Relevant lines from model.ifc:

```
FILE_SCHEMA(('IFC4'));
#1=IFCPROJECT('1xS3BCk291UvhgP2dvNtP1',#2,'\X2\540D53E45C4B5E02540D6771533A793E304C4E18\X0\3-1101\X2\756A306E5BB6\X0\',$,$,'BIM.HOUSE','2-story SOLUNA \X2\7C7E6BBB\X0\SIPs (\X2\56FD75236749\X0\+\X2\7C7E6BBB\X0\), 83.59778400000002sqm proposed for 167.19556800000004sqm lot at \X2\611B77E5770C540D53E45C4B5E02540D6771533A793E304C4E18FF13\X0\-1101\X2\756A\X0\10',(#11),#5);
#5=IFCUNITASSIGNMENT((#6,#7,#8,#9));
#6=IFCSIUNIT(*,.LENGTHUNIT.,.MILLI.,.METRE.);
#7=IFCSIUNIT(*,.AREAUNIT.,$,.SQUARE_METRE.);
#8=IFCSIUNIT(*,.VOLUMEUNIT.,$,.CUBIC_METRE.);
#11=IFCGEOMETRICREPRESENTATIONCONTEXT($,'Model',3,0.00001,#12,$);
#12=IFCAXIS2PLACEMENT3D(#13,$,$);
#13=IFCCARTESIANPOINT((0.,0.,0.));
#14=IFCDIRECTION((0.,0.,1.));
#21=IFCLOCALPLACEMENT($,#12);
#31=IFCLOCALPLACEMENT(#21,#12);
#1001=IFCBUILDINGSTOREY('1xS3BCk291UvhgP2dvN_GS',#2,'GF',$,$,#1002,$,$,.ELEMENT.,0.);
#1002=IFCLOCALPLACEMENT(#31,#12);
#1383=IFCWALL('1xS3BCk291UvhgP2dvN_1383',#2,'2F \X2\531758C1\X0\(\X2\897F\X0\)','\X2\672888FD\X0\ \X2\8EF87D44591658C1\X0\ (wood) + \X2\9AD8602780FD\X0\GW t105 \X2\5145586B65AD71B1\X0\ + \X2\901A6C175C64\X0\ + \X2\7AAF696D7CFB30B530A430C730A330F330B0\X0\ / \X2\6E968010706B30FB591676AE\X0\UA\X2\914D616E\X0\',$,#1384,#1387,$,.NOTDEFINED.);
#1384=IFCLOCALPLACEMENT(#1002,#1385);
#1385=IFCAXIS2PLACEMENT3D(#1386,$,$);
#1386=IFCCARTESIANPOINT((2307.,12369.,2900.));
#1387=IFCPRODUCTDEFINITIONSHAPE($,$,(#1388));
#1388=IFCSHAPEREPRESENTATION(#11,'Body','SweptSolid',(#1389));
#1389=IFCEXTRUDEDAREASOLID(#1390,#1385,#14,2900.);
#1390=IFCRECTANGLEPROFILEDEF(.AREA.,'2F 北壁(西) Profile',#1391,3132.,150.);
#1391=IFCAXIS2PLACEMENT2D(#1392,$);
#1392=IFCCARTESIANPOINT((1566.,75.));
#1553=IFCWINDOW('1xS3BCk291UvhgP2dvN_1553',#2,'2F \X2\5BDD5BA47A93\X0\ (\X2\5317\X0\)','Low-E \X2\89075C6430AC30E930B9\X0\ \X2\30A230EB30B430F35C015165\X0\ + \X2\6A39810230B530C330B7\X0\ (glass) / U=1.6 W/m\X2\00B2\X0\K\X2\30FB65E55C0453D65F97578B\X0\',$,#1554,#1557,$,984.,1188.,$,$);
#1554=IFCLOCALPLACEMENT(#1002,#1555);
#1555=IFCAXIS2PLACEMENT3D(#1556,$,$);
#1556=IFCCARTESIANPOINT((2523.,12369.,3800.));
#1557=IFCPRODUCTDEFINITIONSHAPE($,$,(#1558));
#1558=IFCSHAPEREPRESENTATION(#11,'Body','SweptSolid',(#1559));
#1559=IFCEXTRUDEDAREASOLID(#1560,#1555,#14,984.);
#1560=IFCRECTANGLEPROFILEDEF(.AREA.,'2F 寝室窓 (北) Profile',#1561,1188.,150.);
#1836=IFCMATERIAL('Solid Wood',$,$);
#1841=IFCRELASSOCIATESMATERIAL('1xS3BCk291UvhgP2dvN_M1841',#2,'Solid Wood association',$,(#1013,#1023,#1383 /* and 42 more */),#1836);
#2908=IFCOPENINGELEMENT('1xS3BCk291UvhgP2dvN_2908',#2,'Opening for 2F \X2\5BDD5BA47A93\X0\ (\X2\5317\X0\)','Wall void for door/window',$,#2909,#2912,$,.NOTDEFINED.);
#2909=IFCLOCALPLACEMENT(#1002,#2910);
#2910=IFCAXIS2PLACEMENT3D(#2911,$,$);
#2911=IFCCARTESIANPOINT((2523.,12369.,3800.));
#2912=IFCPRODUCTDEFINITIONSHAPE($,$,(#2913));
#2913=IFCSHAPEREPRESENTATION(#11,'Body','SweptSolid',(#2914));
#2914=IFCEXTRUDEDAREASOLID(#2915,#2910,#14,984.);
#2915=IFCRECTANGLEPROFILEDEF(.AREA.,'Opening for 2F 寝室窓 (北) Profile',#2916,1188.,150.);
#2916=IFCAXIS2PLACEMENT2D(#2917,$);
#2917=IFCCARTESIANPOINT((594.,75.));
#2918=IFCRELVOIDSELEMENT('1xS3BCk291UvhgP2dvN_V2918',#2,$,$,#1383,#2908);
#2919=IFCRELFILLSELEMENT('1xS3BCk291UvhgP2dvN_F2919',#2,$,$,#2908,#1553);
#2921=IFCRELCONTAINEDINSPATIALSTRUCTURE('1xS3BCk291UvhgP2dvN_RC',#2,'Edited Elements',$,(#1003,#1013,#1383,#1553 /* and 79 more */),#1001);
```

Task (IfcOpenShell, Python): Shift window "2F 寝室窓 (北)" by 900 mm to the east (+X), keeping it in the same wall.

```python
import ifcopenshell
import ifcopenshell.api.geometry
import ifcopenshell.util.placement

model = ifcopenshell.open("model.ifc")

window = model.by_guid("1xS3BCk291UvhgP2dvN_1553")
opening = window.FillsVoids[0].RelatingOpeningElement
wall = opening.VoidsElements[0].RelatingBuildingElement

wall_matrix = ifcopenshell.util.placement.get_local_placement(wall.ObjectPlacement)
shift = wall_matrix[:3, 0] * 900.0
before = ifcopenshell.util.placement.get_local_placement(window.ObjectPlacement)[:3, 3].copy()

# The window is not placed relative to its opening, so move both.
for product in (opening, window):
    matrix = ifcopenshell.util.placement.get_local_placement(product.ObjectPlacement)
    matrix[:3, 3] += shift
    ifcopenshell.api.geometry.edit_object_placement(model, product=product, matrix=matrix, is_si=False)

after = ifcopenshell.util.placement.get_local_placement(window.ObjectPlacement)[:3, 3]
print("window moved by", (after - before).round(3) + 0.0)

model.write("model_rev.ifc")
```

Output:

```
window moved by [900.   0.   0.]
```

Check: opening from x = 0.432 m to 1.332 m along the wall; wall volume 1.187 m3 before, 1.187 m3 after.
